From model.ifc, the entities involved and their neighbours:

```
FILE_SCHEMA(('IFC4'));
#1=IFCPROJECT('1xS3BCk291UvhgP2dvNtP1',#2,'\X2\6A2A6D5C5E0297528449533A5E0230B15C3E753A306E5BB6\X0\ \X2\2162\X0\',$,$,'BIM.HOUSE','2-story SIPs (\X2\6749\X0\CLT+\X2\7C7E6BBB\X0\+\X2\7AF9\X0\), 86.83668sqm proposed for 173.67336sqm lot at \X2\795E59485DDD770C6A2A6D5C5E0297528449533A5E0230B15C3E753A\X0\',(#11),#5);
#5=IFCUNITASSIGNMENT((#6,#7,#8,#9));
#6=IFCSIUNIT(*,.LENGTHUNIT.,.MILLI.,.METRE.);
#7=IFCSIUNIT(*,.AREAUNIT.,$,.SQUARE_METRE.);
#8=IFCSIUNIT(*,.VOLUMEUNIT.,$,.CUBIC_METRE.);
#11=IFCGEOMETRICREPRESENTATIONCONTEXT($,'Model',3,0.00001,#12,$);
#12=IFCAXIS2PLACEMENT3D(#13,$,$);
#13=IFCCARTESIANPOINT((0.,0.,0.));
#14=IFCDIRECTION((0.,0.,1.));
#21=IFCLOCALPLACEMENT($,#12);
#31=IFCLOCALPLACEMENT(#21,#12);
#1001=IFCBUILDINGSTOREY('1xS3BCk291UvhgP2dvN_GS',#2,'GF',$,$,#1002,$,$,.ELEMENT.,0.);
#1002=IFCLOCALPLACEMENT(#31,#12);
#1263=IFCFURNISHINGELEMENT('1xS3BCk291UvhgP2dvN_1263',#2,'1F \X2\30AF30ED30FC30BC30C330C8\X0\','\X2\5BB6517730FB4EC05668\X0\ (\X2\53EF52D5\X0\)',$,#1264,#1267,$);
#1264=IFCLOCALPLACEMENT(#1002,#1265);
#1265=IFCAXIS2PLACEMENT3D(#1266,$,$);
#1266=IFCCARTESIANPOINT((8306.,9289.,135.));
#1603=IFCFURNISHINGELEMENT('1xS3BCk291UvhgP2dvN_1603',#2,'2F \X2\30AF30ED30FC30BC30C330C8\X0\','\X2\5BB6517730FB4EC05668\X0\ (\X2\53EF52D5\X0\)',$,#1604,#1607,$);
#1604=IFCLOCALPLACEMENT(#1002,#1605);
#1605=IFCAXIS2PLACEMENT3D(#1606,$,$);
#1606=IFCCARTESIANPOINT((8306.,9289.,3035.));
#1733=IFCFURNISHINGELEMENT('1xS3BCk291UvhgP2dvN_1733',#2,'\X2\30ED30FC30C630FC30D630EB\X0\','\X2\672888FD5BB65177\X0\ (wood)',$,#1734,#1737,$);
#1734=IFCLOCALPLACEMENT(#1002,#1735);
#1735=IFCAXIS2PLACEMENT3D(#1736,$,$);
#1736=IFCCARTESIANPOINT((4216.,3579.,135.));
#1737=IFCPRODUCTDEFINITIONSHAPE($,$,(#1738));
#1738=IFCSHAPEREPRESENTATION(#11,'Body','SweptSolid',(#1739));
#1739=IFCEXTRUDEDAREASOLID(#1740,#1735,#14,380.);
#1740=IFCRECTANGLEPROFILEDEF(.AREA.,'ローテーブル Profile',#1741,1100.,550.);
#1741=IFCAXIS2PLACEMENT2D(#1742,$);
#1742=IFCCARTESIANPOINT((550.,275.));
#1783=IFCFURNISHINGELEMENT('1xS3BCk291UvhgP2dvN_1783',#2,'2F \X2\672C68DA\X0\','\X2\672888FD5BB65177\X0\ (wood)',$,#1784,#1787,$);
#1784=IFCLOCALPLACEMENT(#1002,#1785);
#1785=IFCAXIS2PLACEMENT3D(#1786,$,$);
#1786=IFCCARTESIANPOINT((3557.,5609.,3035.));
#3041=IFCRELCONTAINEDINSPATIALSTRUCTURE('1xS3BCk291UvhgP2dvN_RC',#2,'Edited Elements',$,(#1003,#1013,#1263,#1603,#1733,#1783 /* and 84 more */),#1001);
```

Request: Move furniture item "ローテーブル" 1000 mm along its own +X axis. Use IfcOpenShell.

```python
import ifcopenshell
import ifcopenshell.api.geometry
import ifcopenshell.util.placement
import ifcopenshell.util.unit

model = ifcopenshell.open("model.ifc")
unit_scale = ifcopenshell.util.unit.calculate_unit_scale(model)

item = model.by_guid("1xS3BCk291UvhgP2dvN_1733")
matrix = ifcopenshell.util.placement.get_local_placement(item.ObjectPlacement)
matrix[:3, 3] += matrix[:3, 0] * 1 / unit_scale
ifcopenshell.api.geometry.edit_object_placement(model, product=item, matrix=matrix, is_si=False)

print(ifcopenshell.util.placement.get_local_placement(item.ObjectPlacement).round(3) + 0.0)

model.write("model_rev.ifc")
```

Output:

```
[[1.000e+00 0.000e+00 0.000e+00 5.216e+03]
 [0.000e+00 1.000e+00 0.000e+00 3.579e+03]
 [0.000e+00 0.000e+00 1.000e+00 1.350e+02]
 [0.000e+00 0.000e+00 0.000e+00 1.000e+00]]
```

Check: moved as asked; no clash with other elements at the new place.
